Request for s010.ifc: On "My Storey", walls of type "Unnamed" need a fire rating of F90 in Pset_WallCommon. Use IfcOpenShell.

First a look at what the model holds.

```python
import ifcopenshell
import ifcopenshell.util.element

model = ifcopenshell.open("s010.ifc")
print(model.schema)
storey = next(s for s in model.by_type("IfcBuildingStorey") if s.Name == "My Storey")
walls = [e for e in ifcopenshell.util.element.get_decomposition(storey) if e.is_a("IfcWall")]
seen = {}
for e in walls:
    element_type = ifcopenshell.util.element.get_type(e)
    key = (element_type.Name if element_type != e and element_type else None, ifcopenshell.util.element.get_pset(e, "Pset_WallCommon", "FireRating"))
    seen[key] = seen.get(key, 0) + 1
for (name, value), count in sorted(seen.items(), key=str):
    print(count, "x", name, "|", value)
```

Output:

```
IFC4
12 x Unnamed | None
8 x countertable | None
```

```python
import ifcopenshell
import ifcopenshell.api.pset
import ifcopenshell.util.element

model = ifcopenshell.open("s010.ifc")

storey = next(s for s in model.by_type("IfcBuildingStorey") if s.Name == "My Storey")
walls = [e for e in ifcopenshell.util.element.get_decomposition(storey) if e.is_a("IfcWall")]

count = 0
for e in walls:
    element_type = ifcopenshell.util.element.get_type(e)
    if element_type in (None, e) or element_type.Name != "Unnamed":
        continue
    # add_pset returns the element's existing set when there is one.
    pset = ifcopenshell.api.pset.add_pset(model, product=e, name="Pset_WallCommon")
    ifcopenshell.api.pset.edit_pset(model, pset=pset, properties={"FireRating": "F90"})
    count += 1

print(count, "walls updated")

model.write("s010_rev.ifc")
```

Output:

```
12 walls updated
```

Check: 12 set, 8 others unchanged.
